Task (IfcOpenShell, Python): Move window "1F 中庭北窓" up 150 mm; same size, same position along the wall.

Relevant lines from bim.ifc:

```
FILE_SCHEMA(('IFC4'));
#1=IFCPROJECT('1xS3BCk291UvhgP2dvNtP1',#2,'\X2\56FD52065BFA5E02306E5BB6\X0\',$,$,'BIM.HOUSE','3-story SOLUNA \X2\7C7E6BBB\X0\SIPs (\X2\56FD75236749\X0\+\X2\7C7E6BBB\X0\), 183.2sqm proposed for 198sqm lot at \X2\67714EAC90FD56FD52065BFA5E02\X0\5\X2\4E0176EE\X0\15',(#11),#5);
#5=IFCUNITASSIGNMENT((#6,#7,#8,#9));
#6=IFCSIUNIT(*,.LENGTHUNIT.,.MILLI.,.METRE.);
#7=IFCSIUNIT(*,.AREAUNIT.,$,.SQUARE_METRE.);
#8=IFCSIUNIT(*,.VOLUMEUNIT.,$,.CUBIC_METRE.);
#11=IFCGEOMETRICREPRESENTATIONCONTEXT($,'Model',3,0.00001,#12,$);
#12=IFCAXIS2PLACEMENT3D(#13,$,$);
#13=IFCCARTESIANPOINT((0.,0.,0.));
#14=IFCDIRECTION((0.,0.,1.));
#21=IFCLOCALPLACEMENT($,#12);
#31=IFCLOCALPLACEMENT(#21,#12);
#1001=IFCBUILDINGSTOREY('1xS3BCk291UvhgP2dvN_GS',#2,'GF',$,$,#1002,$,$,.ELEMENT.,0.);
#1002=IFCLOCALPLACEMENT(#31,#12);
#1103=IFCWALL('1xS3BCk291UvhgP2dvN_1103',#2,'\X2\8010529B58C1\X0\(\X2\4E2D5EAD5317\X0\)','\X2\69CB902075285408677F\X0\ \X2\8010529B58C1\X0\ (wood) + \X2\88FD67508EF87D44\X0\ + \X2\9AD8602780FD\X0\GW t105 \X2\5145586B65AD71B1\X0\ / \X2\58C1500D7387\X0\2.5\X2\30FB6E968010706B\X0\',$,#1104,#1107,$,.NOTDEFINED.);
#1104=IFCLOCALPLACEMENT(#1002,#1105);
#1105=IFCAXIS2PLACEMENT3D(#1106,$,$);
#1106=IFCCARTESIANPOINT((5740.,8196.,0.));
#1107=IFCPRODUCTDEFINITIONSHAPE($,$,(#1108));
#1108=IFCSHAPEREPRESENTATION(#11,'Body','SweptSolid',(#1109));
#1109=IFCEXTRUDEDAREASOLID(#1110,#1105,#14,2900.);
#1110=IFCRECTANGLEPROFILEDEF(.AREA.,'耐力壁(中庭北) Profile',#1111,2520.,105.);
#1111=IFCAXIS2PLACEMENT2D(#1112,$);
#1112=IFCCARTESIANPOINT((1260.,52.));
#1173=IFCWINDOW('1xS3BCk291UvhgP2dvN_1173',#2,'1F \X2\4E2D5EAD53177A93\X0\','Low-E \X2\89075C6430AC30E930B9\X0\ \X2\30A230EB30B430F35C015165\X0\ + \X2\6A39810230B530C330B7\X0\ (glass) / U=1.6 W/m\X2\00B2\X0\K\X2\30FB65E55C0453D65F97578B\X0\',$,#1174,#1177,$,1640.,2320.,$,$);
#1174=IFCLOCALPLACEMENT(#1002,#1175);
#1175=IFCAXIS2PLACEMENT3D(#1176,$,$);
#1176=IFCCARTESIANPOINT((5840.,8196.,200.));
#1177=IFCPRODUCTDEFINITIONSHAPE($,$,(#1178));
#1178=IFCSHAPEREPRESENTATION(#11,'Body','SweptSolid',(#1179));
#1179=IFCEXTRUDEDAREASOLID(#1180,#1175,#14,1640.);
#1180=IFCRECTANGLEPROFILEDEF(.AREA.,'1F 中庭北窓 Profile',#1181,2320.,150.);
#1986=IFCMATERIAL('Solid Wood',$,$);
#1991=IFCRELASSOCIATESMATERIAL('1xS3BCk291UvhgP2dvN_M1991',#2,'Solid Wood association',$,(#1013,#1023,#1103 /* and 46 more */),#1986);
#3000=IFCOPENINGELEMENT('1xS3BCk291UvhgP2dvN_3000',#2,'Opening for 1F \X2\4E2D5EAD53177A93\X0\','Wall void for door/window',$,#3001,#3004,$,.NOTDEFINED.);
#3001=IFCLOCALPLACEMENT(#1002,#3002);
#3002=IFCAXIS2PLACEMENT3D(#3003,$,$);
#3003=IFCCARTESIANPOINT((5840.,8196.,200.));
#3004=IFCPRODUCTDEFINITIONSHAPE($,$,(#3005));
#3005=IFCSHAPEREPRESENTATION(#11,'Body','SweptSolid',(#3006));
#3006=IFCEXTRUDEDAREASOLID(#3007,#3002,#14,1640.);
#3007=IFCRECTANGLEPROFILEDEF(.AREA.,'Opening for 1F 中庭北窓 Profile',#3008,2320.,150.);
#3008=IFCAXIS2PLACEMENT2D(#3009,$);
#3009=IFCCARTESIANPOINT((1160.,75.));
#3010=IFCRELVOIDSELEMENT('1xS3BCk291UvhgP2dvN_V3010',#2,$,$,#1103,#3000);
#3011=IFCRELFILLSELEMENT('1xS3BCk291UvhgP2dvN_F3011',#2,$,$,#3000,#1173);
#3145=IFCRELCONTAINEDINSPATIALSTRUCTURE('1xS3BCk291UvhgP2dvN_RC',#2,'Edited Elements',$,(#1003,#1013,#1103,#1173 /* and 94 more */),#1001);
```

```python
import numpy as np
import ifcopenshell
import ifcopenshell.api.geometry
import ifcopenshell.util.placement
import ifcopenshell.util.unit

model = ifcopenshell.open("bim.ifc")
unit_scale = ifcopenshell.util.unit.calculate_unit_scale(model)

window = model.by_guid("1xS3BCk291UvhgP2dvN_1173")
opening = window.FillsVoids[0].RelatingOpeningElement
dz = 0.15 / unit_scale

shift = np.array([0.0, 0.0, dz])
# The window is not placed relative to its opening, so move both.
for product in (opening, window):
    matrix = ifcopenshell.util.placement.get_local_placement(product.ObjectPlacement)
    matrix[:3, 3] += shift
    ifcopenshell.api.geometry.edit_object_placement(model, product=product, matrix=matrix, is_si=False)

print(f"moved by {dz * unit_scale:+.3f} m")

model.write("bim-out.ifc")
```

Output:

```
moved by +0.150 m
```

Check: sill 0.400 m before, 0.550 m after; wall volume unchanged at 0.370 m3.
